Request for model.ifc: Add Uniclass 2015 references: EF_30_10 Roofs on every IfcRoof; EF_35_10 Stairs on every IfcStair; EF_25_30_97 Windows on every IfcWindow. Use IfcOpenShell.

First a look at what the model holds.

```python
import ifcopenshell

model = ifcopenshell.open("model.ifc")
print(model.schema)
print("classifications:", [c.Name for c in model.by_type("IfcClassification")])
for ifc_class in ("IfcDoor", "IfcRoof", "IfcStair", "IfcWall", "IfcWindow"):
    print(ifc_class, len(model.by_type(ifc_class)))
```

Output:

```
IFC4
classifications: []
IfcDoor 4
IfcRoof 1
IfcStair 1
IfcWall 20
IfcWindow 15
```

```python
import ifcopenshell
import ifcopenshell.api.classification

model = ifcopenshell.open("model.ifc")

system = ifcopenshell.api.classification.add_classification(model, classification="Uniclass 2015")

codes = {
    "IfcRoof": ("EF_30_10", "Roofs"),
    "IfcStair": ("EF_35_10", "Stairs"),
    "IfcWindow": ("EF_25_30_97", "Windows"),
}
for ifc_class, (code, name) in codes.items():
    products = model.by_type(ifc_class)
    ifcopenshell.api.classification.add_reference(
        model, products=products, classification=system, identification=code, name=name
    )
    print(code, len(products))

model.write("model_updated.ifc")
```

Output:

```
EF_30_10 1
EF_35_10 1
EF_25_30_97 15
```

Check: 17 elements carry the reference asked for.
